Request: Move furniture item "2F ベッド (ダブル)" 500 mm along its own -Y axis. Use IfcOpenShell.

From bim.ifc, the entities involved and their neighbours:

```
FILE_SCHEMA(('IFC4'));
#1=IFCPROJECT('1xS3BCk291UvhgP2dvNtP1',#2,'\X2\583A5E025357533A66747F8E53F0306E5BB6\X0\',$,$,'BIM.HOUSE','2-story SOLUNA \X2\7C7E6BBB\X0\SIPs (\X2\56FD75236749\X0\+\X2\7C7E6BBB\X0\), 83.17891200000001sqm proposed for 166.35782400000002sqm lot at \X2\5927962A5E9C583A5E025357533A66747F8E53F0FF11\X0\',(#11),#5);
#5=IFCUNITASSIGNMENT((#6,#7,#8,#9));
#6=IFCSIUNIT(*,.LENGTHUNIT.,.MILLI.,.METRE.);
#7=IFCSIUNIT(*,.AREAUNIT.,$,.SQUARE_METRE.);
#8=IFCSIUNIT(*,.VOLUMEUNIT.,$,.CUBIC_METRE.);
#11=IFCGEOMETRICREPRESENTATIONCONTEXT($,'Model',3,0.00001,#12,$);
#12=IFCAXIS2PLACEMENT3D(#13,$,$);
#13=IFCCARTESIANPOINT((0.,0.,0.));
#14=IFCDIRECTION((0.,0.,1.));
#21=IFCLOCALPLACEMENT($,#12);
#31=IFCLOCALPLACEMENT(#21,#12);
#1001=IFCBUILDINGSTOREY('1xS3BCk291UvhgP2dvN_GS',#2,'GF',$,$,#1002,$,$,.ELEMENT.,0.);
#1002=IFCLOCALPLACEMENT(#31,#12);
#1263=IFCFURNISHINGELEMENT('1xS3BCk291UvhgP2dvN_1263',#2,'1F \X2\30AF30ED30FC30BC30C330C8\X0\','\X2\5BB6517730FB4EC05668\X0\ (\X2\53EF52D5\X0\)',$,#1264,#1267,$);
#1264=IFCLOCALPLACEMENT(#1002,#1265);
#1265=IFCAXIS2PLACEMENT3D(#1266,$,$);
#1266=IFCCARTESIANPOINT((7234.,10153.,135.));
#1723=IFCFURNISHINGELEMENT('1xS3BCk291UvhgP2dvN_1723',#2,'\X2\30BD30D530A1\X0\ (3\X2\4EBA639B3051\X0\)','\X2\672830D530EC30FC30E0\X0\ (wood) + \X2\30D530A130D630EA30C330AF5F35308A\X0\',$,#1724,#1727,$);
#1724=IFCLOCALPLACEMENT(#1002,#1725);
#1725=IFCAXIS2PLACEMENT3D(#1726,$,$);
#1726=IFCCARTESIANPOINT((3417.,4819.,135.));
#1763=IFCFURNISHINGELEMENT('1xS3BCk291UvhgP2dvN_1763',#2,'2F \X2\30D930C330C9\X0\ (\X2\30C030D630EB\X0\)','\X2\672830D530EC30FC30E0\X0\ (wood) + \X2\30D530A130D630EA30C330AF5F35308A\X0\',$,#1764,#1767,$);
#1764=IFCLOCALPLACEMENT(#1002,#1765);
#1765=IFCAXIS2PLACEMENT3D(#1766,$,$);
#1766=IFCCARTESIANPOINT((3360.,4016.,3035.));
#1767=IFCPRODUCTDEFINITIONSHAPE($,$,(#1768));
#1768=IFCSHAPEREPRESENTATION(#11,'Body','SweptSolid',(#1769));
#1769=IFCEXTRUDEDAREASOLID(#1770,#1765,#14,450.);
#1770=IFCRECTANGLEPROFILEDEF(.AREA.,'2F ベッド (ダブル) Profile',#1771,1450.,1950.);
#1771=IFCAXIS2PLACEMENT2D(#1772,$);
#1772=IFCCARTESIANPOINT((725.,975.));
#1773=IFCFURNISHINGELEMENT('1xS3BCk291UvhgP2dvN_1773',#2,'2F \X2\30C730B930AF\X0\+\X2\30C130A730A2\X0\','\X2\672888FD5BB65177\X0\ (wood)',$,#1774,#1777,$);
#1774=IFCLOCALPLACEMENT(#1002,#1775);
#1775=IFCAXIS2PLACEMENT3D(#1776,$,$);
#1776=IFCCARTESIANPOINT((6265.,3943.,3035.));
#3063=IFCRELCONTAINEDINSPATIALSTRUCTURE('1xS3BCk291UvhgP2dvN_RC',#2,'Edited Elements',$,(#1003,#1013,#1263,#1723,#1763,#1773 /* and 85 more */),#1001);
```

```python
import ifcopenshell
import ifcopenshell.api.geometry
import ifcopenshell.util.placement

model = ifcopenshell.open("bim.ifc")

item = model.by_id(1763)
matrix = ifcopenshell.util.placement.get_local_placement(item.ObjectPlacement)
matrix[:3, 3] -= matrix[:3, 1] * 500.0
ifcopenshell.api.geometry.edit_object_placement(model, product=item, matrix=matrix, is_si=False)

print(ifcopenshell.util.placement.get_local_placement(item.ObjectPlacement).round(3) + 0.0)

model.write("bim_updated.ifc")
```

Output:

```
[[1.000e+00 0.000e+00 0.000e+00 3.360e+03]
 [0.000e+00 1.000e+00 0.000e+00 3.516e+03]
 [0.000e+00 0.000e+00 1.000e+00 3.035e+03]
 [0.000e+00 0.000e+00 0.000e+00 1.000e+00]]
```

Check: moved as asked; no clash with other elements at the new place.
